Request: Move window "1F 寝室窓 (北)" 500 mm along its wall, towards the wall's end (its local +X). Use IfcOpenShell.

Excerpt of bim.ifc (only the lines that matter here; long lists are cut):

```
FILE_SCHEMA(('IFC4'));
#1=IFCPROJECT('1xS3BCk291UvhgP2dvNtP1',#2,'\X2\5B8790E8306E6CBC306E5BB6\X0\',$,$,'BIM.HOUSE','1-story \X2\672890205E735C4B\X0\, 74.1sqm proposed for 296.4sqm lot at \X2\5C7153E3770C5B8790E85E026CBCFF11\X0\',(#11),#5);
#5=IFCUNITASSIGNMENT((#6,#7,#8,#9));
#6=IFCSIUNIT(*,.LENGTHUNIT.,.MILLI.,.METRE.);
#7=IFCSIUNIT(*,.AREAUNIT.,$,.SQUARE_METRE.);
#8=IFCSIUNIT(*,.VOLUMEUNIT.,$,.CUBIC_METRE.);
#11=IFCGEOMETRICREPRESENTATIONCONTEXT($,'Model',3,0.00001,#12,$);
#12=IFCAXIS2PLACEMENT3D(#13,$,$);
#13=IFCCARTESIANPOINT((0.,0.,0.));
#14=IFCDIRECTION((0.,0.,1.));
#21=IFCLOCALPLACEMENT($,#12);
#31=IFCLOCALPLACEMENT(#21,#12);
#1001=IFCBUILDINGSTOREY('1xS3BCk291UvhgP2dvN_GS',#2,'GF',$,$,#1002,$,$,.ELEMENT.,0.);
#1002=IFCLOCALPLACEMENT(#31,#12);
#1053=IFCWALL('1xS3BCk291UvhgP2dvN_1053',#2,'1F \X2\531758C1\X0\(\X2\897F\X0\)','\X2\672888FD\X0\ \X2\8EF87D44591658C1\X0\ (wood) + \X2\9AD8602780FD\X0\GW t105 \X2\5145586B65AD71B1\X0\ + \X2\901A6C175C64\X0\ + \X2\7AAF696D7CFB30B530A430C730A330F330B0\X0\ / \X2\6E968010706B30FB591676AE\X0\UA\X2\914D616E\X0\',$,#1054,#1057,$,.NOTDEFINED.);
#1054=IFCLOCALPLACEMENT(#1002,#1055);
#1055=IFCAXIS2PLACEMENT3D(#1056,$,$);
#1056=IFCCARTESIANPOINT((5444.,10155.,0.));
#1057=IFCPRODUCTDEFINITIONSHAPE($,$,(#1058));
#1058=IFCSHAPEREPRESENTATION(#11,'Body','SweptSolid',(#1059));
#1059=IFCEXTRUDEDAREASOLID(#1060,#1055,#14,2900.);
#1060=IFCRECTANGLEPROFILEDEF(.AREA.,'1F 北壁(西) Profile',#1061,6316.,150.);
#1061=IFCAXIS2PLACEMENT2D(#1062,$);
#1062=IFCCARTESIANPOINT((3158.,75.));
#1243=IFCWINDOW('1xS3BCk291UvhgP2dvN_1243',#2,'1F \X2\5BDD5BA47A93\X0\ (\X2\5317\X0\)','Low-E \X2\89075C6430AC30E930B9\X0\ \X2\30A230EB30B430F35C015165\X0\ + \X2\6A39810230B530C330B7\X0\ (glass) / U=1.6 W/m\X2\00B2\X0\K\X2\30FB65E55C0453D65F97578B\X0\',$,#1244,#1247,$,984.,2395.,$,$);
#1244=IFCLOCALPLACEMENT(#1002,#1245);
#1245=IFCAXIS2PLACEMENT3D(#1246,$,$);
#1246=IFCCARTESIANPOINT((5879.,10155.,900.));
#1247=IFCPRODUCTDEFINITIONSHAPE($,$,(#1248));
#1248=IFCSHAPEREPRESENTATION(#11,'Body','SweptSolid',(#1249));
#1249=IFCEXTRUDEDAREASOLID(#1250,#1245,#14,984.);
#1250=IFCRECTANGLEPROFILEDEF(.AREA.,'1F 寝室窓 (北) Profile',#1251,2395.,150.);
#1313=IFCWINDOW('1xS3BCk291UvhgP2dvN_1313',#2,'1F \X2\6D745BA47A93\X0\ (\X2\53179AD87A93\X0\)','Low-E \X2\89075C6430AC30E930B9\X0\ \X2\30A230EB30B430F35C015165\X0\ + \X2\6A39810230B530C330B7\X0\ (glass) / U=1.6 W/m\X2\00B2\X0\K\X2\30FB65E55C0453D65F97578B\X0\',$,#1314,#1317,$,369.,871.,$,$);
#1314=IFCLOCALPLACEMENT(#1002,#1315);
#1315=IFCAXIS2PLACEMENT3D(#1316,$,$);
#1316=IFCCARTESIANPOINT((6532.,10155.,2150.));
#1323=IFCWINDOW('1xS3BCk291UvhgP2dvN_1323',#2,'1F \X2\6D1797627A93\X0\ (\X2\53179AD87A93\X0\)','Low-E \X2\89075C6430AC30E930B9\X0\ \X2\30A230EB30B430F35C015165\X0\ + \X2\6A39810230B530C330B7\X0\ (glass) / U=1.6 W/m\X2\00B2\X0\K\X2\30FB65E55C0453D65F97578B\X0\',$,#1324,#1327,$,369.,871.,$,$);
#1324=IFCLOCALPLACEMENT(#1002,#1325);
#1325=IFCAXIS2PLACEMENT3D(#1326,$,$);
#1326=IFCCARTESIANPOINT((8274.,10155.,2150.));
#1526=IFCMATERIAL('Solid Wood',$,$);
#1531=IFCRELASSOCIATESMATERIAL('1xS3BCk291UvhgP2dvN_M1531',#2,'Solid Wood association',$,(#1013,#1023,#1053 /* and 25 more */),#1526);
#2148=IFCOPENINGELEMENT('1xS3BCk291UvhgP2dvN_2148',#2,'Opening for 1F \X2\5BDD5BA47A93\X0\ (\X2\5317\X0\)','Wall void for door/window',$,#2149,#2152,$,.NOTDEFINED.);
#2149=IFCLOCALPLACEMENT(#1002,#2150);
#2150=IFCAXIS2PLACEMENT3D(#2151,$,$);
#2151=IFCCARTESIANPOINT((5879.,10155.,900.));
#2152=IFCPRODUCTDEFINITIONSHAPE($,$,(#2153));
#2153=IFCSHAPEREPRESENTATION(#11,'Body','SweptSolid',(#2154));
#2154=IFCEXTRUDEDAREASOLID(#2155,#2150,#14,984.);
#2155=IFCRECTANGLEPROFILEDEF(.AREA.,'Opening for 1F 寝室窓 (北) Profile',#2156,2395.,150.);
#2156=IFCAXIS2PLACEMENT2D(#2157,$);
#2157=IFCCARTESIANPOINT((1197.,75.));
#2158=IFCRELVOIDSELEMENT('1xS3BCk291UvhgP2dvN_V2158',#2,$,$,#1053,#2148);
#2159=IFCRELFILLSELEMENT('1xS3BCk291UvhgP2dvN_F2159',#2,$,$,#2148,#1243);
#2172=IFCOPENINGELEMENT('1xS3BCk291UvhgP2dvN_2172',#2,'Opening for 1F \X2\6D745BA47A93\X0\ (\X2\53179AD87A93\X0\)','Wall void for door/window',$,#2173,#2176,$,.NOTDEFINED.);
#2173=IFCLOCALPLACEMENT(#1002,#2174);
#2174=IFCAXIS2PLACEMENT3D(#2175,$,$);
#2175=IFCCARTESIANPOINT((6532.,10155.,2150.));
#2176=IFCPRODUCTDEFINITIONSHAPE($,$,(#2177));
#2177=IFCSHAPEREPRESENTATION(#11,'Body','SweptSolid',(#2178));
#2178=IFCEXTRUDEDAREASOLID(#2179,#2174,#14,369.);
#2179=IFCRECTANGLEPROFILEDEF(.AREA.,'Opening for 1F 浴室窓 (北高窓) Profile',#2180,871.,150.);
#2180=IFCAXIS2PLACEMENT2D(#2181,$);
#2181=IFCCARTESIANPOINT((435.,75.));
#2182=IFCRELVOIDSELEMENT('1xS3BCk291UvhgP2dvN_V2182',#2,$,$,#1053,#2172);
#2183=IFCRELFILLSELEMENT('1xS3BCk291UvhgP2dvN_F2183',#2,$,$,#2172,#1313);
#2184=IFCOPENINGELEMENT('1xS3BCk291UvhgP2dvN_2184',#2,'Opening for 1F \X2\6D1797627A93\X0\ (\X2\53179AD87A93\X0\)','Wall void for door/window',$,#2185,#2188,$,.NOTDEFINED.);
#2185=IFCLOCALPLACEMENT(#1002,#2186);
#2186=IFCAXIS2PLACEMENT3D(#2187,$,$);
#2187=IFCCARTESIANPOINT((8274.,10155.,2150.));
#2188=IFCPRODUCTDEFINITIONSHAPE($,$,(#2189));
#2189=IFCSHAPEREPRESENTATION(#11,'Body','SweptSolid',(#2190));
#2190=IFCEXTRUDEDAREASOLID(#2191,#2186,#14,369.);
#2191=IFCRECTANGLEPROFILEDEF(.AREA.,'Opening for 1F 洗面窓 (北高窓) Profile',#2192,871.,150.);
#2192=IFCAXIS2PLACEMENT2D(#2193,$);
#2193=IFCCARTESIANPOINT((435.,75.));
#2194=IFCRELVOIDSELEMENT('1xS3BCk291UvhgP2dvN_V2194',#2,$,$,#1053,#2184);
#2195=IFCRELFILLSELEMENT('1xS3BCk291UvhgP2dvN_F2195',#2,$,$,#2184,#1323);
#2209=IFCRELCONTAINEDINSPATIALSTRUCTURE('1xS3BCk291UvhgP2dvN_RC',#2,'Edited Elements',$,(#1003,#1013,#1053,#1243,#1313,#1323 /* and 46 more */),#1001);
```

```python
import ifcopenshell
import ifcopenshell.api.geometry
import ifcopenshell.util.placement
import ifcopenshell.util.unit

model = ifcopenshell.open("bim.ifc")
unit_scale = ifcopenshell.util.unit.calculate_unit_scale(model)

window = model.by_guid("1xS3BCk291UvhgP2dvN_1243")
opening = window.FillsVoids[0].RelatingOpeningElement
wall = opening.VoidsElements[0].RelatingBuildingElement

wall_matrix = ifcopenshell.util.placement.get_local_placement(wall.ObjectPlacement)
shift = wall_matrix[:3, 0] * 0.5 / unit_scale
before = ifcopenshell.util.placement.get_local_placement(window.ObjectPlacement)[:3, 3].copy()

# The window is not placed relative to its opening, so move both.
for product in (opening, window):
    matrix = ifcopenshell.util.placement.get_local_placement(product.ObjectPlacement)
    matrix[:3, 3] += shift
    ifcopenshell.api.geometry.edit_object_placement(model, product=product, matrix=matrix, is_si=False)

after = ifcopenshell.util.placement.get_local_placement(window.ObjectPlacement)[:3, 3]
print("window moved by", (after - before).round(3) + 0.0)

model.write("bim-out.ifc")
```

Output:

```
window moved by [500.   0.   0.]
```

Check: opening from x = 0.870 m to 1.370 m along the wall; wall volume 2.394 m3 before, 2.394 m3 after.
